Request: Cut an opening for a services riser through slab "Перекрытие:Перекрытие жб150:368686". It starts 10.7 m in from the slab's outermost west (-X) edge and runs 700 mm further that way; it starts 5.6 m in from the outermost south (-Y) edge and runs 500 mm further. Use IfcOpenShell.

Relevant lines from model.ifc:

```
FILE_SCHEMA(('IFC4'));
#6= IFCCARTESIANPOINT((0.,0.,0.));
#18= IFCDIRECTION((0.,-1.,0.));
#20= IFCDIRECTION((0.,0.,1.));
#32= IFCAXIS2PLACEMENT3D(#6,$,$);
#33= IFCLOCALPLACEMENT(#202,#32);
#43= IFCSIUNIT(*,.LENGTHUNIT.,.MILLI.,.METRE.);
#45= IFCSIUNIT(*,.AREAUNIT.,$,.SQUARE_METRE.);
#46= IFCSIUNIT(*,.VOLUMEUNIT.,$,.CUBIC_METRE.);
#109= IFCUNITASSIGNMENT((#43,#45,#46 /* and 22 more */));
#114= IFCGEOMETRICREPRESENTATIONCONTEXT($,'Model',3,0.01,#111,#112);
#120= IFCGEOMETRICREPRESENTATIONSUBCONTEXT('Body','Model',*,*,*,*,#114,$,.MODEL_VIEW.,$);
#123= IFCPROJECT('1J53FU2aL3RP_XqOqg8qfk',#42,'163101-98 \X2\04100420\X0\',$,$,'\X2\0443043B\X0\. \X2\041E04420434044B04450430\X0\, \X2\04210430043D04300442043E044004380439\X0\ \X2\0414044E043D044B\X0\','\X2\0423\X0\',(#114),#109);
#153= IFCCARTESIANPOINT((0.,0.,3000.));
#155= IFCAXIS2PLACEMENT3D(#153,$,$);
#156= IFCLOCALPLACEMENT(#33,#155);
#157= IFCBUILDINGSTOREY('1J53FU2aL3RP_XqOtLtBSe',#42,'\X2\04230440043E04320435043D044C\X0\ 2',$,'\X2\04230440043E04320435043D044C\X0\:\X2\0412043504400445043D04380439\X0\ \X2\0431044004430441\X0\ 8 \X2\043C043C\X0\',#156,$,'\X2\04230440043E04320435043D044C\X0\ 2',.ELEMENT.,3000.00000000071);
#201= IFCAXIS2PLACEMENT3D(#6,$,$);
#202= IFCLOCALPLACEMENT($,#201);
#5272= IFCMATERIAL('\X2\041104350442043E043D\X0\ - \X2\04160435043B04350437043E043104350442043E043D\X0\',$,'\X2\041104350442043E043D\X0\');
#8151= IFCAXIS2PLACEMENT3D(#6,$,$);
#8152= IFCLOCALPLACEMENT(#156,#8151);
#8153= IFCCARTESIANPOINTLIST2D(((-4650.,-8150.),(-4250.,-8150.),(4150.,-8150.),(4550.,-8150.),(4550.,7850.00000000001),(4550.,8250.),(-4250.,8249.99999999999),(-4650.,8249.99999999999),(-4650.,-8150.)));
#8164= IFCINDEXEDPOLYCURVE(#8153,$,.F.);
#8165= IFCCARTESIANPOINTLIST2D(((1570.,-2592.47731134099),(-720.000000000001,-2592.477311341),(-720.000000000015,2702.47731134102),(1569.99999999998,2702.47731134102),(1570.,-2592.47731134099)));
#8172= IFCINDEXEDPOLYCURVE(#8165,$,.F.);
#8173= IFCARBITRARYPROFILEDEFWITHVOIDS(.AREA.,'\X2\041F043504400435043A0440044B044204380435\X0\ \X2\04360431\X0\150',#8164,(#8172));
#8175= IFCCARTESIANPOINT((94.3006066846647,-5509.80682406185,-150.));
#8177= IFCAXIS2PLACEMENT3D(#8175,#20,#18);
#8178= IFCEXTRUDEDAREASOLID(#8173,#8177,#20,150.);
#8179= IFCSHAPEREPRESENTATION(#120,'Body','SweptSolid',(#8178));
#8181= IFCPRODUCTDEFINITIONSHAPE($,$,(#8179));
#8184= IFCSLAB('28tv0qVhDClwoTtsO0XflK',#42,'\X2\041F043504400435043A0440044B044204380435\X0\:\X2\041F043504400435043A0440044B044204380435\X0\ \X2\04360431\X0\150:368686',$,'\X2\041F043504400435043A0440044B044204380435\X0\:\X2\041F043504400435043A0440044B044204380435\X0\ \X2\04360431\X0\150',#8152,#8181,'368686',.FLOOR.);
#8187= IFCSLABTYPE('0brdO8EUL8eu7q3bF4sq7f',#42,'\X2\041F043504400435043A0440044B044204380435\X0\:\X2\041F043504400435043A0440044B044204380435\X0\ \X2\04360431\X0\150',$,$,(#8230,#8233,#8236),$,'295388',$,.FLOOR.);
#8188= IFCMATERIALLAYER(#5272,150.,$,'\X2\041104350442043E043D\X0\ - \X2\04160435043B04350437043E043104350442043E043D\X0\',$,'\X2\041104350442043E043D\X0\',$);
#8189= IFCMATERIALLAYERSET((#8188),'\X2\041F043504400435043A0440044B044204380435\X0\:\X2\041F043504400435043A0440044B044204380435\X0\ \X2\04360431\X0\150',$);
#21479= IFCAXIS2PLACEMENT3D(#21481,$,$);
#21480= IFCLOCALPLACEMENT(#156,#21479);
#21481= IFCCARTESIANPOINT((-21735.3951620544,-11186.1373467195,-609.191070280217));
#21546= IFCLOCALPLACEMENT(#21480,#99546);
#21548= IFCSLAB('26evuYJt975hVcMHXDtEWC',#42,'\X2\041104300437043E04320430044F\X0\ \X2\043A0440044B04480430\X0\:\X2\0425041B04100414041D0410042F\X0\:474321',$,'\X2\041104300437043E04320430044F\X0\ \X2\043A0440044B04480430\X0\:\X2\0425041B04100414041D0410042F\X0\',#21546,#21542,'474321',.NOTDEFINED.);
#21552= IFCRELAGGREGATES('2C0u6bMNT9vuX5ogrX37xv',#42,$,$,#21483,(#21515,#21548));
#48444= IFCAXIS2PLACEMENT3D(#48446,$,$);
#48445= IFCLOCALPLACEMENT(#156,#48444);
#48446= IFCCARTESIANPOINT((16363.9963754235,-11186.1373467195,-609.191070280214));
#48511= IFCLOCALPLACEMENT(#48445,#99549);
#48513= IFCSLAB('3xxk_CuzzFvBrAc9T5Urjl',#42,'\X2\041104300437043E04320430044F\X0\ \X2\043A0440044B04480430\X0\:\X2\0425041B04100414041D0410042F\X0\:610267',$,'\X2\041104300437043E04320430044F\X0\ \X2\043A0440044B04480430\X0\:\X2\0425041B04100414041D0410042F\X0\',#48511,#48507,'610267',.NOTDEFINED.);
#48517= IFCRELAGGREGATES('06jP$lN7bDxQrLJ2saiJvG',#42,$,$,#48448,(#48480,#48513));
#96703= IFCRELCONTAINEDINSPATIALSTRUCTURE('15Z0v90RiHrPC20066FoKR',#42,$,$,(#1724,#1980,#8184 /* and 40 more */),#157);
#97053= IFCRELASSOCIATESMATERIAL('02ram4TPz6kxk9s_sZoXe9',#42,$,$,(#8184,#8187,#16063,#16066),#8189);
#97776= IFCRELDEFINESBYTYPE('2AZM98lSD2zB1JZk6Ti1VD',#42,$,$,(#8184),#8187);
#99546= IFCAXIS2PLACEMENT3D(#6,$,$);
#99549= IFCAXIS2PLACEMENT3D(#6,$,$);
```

```python
import numpy as np
import ifcopenshell
import ifcopenshell.api.feature
import ifcopenshell.api.geometry
import ifcopenshell.api.root
import ifcopenshell.geom
import ifcopenshell.util.placement
import ifcopenshell.util.representation
import ifcopenshell.util.shape
import ifcopenshell.util.unit

model = ifcopenshell.open("model.ifc")
unit_scale = ifcopenshell.util.unit.calculate_unit_scale(model)
settings = ifcopenshell.geom.settings()


def volume(element):
    """Net volume in cubic metres, openings subtracted."""
    shape = ifcopenshell.geom.create_shape(settings, element)
    return ifcopenshell.util.shape.get_volume(shape.geometry)


slab = model.by_id(8184)
before = volume(slab)

# Extent in the slab's own axes, in metres. The edges named are its -X and -Y sides.
slab_shape = ifcopenshell.geom.create_shape(settings, slab)
vertices = ifcopenshell.util.shape.get_vertices(slab_shape.geometry)
x_min, y_min, bottom = vertices.min(axis=0)
top = vertices[:, 2].max()

opening = ifcopenshell.api.root.create_entity(model, ifc_class="IfcOpeningElement", name="Services riser opening", predefined_type="OPENING")
context = ifcopenshell.util.representation.get_context(model, "Model", "Body", "MODEL_VIEW")
width, depth = 0.7, 0.5
outline = [(0.0, 0.0), (width, 0.0), (width, depth), (0.0, depth), (0.0, 0.0)]
# Overshoot both faces by 50 mm so the cut is clean.
shape = ifcopenshell.api.geometry.add_slab_representation(
    model, context=context, depth=top - bottom + 0.1, polyline=outline
)
ifcopenshell.api.geometry.assign_representation(model, product=opening, representation=shape)

matrix = ifcopenshell.util.placement.get_local_placement(slab.ObjectPlacement)
matrix[:, 3] = matrix @ np.append(np.array([x_min + 10.7, y_min + 5.6, bottom - 0.05]) / unit_scale, 1.0)
ifcopenshell.api.geometry.edit_object_placement(model, product=opening, matrix=matrix, is_si=False)
ifcopenshell.api.feature.add_feature(model, feature=opening, element=slab)

after = volume(slab)

print(f"slab volume {before:.3f} -> {after:.3f} m3")

model.write("model_updated.ifc")
```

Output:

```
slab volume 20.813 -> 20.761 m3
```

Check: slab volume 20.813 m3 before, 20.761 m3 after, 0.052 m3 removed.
